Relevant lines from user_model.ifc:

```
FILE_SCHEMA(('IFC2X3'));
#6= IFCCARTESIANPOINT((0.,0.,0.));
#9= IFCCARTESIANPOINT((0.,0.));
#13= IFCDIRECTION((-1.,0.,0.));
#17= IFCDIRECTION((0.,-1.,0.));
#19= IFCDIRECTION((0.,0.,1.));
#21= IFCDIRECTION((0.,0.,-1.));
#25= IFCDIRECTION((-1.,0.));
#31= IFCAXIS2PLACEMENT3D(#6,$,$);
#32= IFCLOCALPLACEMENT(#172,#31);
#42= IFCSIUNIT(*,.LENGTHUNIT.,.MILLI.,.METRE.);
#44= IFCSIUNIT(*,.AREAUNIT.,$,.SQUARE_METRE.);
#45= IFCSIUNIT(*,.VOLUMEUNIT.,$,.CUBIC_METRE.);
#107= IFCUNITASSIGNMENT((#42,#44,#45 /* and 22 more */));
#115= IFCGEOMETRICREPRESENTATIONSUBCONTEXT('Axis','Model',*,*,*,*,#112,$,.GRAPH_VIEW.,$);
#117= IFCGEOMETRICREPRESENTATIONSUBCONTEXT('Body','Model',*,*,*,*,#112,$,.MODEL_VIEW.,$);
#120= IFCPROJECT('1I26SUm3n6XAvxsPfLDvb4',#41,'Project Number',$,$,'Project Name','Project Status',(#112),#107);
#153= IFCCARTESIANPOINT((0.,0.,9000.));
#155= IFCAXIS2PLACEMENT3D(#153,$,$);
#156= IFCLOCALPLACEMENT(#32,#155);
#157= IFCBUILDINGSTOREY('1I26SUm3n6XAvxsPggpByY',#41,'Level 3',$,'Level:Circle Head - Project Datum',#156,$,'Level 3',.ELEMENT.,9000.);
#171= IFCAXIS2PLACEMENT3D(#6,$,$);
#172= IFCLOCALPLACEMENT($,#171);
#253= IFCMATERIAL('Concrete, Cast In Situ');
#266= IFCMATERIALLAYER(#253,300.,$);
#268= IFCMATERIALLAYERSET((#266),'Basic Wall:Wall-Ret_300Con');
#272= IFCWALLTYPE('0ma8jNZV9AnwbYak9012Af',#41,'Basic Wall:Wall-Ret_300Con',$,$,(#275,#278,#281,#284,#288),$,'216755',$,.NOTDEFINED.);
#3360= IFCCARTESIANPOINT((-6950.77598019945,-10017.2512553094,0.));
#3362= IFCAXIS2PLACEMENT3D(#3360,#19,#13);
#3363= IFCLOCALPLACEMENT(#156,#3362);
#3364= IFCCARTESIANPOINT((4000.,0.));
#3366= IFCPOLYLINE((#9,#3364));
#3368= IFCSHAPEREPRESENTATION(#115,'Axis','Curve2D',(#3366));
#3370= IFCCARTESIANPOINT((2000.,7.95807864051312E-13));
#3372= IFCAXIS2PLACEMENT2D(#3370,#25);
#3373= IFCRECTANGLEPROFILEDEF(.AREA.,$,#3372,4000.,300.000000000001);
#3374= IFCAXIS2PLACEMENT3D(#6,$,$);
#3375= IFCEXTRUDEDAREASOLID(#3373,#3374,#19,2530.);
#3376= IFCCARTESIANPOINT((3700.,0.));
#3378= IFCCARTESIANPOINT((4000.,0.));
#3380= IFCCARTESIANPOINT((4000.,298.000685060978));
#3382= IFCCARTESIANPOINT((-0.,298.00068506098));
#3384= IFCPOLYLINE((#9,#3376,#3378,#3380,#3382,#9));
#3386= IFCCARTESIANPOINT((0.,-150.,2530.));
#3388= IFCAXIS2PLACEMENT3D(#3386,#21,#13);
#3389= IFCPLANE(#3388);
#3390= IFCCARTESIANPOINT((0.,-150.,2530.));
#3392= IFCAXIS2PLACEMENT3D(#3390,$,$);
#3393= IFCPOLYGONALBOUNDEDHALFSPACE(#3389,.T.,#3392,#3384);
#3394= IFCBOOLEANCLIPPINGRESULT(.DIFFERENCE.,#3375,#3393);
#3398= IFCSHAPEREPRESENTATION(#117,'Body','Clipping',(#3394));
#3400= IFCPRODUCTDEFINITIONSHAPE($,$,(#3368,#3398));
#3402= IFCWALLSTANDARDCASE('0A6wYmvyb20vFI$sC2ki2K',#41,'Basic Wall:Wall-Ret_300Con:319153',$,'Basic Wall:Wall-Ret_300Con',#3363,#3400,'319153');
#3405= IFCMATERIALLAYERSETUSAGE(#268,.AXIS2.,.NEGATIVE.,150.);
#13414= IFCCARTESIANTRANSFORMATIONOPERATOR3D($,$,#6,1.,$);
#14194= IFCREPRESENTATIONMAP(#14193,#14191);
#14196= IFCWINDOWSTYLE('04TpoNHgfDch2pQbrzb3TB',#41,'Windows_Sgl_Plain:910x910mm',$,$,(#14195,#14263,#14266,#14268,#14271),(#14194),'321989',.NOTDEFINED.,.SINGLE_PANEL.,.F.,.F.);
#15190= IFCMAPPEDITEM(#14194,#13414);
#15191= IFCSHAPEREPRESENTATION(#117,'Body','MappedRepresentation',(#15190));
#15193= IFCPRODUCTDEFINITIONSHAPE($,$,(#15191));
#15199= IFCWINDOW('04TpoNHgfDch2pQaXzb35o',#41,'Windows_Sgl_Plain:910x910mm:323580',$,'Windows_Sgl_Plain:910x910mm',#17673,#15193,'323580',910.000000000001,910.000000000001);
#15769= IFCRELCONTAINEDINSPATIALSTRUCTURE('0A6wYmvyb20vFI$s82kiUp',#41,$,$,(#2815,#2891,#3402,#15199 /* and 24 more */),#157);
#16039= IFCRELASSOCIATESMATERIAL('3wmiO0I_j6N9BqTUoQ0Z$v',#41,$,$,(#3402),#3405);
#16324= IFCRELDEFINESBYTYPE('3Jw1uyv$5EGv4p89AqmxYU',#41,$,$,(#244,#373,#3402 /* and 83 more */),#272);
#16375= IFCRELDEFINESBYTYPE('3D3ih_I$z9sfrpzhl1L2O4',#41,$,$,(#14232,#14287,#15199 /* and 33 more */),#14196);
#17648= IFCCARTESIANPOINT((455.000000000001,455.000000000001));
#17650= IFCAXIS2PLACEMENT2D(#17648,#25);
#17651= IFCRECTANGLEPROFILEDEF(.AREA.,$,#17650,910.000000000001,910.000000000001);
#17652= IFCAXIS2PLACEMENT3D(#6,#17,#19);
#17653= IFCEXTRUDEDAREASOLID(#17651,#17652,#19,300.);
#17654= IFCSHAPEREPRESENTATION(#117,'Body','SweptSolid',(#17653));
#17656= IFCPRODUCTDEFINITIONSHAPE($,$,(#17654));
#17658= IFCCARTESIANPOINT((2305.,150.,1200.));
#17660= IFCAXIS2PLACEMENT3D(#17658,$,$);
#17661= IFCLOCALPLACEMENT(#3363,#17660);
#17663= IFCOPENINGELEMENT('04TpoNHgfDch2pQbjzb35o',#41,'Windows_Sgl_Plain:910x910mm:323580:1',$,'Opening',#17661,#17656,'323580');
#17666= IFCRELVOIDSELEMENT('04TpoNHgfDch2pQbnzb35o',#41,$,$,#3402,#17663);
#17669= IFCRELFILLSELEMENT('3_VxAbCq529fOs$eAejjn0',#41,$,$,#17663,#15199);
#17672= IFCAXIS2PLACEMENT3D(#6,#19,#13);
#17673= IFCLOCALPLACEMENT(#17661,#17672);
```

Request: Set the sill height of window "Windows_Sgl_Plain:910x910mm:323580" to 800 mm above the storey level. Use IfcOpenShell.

```python
import numpy as np
import ifcopenshell
import ifcopenshell.api.geometry
import ifcopenshell.geom
import ifcopenshell.util.element
import ifcopenshell.util.placement
import ifcopenshell.util.shape
import ifcopenshell.util.unit

model = ifcopenshell.open("user_model.ifc")
unit_scale = ifcopenshell.util.unit.calculate_unit_scale(model)

window = model.by_guid("04TpoNHgfDch2pQaXzb35o")
opening = window.FillsVoids[0].RelatingOpeningElement
storey = ifcopenshell.util.element.get_container(window, ifc_class="IfcBuildingStorey")
level = ifcopenshell.util.placement.get_local_placement(storey.ObjectPlacement)[2, 3]

# The opening's origin need not be at the sill, so measure its lowest point.
shape = ifcopenshell.geom.create_shape(ifcopenshell.geom.settings(), opening)
bottom = ifcopenshell.util.shape.get_shape_bottom_elevation(shape, shape.geometry) / unit_scale
dz = level + 0.8 / unit_scale - bottom

shift = np.array([0.0, 0.0, dz])
# The window is placed relative to its opening, so it follows when the opening moves.
matrix = ifcopenshell.util.placement.get_local_placement(opening.ObjectPlacement)
matrix[:3, 3] += shift
ifcopenshell.api.geometry.edit_object_placement(
    model, product=opening, matrix=matrix, is_si=False, should_transform_children=True
)

print(f"moved by {dz * unit_scale:+.3f} m")

model.write("user_model-out.ifc")
```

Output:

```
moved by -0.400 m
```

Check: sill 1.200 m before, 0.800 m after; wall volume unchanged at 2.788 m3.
